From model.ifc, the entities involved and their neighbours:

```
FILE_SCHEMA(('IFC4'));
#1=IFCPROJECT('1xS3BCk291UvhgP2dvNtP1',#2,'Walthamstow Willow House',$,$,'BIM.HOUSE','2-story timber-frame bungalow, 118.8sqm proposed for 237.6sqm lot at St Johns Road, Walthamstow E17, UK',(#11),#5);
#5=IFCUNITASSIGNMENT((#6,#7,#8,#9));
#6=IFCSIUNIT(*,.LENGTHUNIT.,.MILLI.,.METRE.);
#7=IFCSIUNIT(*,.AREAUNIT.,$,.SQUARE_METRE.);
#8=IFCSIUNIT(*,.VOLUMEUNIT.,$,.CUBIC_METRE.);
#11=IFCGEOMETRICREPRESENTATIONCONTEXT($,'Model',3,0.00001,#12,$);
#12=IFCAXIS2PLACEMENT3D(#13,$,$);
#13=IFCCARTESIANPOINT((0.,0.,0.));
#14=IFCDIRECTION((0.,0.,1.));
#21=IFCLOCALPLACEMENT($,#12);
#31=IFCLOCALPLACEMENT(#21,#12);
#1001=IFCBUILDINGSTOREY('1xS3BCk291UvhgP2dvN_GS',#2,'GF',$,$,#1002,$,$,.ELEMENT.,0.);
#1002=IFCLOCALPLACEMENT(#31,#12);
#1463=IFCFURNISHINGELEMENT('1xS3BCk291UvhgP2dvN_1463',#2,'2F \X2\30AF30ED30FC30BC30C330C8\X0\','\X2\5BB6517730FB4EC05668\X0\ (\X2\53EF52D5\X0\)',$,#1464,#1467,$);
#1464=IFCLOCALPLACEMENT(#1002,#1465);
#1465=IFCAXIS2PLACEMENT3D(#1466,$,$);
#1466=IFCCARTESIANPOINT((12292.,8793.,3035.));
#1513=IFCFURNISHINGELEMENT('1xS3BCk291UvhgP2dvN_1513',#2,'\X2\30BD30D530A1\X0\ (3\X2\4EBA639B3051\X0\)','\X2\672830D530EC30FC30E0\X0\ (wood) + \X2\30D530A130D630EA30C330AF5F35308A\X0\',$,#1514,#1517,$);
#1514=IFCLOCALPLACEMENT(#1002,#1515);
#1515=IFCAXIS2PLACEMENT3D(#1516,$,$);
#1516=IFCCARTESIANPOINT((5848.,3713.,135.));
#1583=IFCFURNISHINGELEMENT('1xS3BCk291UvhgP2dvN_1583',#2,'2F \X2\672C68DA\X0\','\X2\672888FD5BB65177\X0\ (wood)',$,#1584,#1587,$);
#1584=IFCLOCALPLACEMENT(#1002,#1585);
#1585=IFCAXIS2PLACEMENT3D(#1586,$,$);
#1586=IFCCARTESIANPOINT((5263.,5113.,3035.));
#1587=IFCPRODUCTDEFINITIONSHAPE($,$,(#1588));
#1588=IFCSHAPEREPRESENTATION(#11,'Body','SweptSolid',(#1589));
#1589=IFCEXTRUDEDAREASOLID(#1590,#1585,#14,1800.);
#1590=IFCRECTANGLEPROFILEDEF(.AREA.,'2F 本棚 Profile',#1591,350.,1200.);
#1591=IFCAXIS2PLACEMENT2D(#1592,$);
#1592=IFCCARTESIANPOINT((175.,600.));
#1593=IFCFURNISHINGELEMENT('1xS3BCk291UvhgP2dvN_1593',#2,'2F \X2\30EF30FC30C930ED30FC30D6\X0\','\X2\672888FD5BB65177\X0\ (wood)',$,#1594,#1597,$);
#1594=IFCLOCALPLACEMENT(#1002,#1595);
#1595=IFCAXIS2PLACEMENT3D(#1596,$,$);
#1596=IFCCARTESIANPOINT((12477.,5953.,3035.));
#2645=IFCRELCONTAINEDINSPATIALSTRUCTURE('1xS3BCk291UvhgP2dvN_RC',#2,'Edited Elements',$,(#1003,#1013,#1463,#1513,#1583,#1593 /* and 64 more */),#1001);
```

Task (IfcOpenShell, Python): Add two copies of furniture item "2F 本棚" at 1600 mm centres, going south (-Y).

```python
import numpy as np
import ifcopenshell
import ifcopenshell.api.geometry
import ifcopenshell.api.root
import ifcopenshell.util.element
import ifcopenshell.util.placement

model = ifcopenshell.open("model.ifc")


def reuse_history(source, copy):
    """copy_class also copies each property set's owner history, people and application; keep the originals."""
    for rel in copy.IsDefinedBy:
        if rel.is_a("IfcRelDefinesByProperties") and (history := rel.RelatingPropertyDefinition.OwnerHistory):
            rel.RelatingPropertyDefinition.OwnerHistory = source.OwnerHistory
            ifcopenshell.util.element.remove_deep2(model, history)


source = model.by_guid("1xS3BCk291UvhgP2dvN_1583")
base = ifcopenshell.util.placement.get_local_placement(source.ObjectPlacement)
step = np.array([0.0, -1.0, 0.0]) * 1600.0

for i in range(1, 3):
    copy = ifcopenshell.api.root.copy_class(model, product=source)
    copy.Representation = ifcopenshell.util.element.copy_deep(
        model, source.Representation, exclude=["IfcGeometricRepresentationContext", "IfcRepresentationMap"]
    )
    reuse_history(source, copy)
    matrix = base.copy()
    matrix[:3, 3] += i * step
    print("added at", matrix[:3, 3].round(3) + 0.0)
    ifcopenshell.api.geometry.edit_object_placement(model, product=copy, matrix=matrix, is_si=False)

model.write("model_edited.ifc")
```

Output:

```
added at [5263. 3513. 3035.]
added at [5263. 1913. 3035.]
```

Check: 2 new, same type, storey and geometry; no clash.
